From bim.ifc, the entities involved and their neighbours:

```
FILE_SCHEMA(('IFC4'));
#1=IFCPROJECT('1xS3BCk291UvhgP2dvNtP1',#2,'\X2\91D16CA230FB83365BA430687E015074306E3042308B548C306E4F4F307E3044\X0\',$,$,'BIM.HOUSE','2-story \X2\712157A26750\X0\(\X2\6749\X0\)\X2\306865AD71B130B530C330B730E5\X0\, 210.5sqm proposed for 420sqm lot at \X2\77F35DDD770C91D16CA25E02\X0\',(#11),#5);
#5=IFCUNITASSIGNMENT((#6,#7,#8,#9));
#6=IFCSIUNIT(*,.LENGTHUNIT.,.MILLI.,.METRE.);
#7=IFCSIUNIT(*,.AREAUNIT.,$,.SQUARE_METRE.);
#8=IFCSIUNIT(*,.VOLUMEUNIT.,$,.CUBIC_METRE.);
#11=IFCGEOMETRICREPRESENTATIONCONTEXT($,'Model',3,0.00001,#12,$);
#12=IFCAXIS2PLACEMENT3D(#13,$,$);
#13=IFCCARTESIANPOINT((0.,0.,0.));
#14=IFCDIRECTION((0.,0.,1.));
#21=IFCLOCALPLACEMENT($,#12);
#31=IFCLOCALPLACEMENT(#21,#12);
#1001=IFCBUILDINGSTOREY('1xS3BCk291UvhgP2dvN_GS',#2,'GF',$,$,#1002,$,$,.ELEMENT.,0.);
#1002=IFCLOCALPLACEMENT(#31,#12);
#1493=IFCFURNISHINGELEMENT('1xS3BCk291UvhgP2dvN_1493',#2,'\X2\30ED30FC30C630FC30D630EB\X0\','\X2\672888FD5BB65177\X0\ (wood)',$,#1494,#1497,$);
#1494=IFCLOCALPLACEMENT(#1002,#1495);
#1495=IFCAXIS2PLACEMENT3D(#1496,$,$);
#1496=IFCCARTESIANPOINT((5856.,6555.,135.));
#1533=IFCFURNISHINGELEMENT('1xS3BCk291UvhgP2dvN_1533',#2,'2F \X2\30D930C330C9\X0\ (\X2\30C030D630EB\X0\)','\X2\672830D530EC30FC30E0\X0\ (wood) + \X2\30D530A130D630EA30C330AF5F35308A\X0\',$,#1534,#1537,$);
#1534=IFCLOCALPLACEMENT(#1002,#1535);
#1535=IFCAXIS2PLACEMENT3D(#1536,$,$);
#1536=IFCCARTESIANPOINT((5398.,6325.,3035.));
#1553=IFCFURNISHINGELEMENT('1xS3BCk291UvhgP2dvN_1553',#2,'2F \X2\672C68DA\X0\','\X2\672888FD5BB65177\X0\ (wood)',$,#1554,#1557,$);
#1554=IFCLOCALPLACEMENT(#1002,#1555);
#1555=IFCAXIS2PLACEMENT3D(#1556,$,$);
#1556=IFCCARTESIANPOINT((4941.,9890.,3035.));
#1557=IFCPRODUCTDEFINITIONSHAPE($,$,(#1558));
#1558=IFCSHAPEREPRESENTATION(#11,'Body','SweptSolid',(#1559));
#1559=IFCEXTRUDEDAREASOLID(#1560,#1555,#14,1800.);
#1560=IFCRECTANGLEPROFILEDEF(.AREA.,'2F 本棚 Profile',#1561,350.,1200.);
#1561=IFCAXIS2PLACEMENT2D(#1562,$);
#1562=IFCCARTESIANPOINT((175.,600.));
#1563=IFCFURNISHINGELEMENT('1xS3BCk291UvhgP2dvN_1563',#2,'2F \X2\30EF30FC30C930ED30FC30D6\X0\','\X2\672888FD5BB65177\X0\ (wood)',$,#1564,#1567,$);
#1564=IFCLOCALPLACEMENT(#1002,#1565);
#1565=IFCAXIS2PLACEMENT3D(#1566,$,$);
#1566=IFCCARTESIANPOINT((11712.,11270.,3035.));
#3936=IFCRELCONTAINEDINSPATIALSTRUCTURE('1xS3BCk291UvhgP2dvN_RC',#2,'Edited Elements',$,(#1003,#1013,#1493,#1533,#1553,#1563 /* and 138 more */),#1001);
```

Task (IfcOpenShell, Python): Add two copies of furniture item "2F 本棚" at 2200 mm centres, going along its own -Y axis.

```python
import ifcopenshell
import ifcopenshell.api.geometry
import ifcopenshell.api.root
import ifcopenshell.util.element
import ifcopenshell.util.placement
import ifcopenshell.util.unit

model = ifcopenshell.open("bim.ifc")
unit_scale = ifcopenshell.util.unit.calculate_unit_scale(model)


def reuse_history(source, copy):
    """copy_class also copies each property set's owner history, people and application; keep the originals."""
    for rel in copy.IsDefinedBy:
        if rel.is_a("IfcRelDefinesByProperties") and (history := rel.RelatingPropertyDefinition.OwnerHistory):
            rel.RelatingPropertyDefinition.OwnerHistory = source.OwnerHistory
            ifcopenshell.util.element.remove_deep2(model, history)


source = model.by_guid("1xS3BCk291UvhgP2dvN_1553")
base = ifcopenshell.util.placement.get_local_placement(source.ObjectPlacement)
step = -base[:3, 1] * 2.2 / unit_scale

for i in range(1, 3):
    copy = ifcopenshell.api.root.copy_class(model, product=source)
    copy.Representation = ifcopenshell.util.element.copy_deep(
        model, source.Representation, exclude=["IfcGeometricRepresentationContext", "IfcRepresentationMap"]
    )
    reuse_history(source, copy)
    matrix = base.copy()
    matrix[:3, 3] += i * step
    print("added at", matrix[:3, 3].round(3) + 0.0)
    ifcopenshell.api.geometry.edit_object_placement(model, product=copy, matrix=matrix, is_si=False)

model.write("bim_updated.ifc")
```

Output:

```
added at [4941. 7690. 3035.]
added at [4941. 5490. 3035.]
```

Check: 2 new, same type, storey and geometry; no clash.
